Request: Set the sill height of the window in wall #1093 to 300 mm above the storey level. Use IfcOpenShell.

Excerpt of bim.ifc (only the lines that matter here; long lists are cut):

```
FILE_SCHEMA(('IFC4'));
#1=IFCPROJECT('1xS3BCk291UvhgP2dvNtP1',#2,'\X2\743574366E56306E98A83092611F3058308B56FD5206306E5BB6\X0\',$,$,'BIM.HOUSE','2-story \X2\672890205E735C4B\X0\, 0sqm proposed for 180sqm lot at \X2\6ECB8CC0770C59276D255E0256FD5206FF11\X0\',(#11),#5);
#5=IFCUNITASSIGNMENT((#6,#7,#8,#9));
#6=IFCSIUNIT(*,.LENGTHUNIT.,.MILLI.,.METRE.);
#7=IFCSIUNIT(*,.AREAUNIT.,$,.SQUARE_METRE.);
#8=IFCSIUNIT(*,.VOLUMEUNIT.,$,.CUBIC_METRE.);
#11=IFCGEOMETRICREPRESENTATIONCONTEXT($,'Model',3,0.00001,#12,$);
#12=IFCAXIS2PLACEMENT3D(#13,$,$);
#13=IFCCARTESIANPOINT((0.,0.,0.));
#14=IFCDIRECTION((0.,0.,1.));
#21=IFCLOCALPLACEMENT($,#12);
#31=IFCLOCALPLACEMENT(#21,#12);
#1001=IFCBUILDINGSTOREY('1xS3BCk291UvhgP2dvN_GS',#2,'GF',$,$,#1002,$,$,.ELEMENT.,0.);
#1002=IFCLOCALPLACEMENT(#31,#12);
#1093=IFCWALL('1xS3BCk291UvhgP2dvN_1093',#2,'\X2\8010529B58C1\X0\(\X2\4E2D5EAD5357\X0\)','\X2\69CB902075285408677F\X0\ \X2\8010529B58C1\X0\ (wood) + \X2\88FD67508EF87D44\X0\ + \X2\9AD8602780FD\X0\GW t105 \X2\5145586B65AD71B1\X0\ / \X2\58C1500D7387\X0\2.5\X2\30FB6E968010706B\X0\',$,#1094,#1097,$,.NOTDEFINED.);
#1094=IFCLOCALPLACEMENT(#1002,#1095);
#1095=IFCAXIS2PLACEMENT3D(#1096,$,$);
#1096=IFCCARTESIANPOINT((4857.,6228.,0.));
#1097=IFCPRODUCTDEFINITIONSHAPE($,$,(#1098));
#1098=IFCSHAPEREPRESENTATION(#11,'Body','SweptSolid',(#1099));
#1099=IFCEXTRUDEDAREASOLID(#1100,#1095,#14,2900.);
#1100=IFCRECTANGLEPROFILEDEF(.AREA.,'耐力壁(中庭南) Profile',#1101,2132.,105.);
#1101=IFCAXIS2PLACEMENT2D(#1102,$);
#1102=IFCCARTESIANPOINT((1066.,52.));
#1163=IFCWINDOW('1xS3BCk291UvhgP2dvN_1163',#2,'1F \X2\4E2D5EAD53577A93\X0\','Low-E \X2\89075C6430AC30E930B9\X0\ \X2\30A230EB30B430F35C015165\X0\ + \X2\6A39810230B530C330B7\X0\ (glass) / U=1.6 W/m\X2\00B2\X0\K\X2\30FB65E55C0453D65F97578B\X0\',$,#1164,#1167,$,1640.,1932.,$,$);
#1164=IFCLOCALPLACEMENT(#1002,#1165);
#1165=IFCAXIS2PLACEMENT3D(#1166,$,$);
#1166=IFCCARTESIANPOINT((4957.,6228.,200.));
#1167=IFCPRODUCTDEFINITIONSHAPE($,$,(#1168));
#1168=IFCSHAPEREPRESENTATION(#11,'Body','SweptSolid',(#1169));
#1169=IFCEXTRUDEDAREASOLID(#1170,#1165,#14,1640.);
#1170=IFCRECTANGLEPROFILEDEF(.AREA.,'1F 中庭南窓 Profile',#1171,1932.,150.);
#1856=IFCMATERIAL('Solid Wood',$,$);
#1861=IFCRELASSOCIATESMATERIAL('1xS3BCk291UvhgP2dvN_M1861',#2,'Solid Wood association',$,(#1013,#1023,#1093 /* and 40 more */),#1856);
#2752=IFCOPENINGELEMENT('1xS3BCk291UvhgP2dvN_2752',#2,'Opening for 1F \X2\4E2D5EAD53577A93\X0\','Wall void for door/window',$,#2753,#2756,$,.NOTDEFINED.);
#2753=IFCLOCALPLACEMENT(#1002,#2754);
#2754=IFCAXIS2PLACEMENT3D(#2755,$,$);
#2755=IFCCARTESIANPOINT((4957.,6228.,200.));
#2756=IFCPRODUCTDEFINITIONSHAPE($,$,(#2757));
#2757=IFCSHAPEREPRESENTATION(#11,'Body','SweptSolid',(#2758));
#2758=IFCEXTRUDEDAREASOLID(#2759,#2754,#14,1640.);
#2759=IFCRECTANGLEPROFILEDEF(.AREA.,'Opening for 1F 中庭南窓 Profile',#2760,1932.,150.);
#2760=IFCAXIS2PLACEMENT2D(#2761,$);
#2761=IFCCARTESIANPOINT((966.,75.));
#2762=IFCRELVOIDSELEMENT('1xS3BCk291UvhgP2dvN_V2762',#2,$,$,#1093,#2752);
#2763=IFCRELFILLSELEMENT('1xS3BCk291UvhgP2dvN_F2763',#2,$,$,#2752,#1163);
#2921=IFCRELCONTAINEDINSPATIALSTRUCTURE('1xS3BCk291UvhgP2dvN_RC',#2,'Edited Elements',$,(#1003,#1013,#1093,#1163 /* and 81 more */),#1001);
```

```python
import numpy as np
import ifcopenshell
import ifcopenshell.api.geometry
import ifcopenshell.geom
import ifcopenshell.util.element
import ifcopenshell.util.placement
import ifcopenshell.util.shape
import ifcopenshell.util.unit

model = ifcopenshell.open("bim.ifc")
unit_scale = ifcopenshell.util.unit.calculate_unit_scale(model)

window = model.by_id(1163)
opening = window.FillsVoids[0].RelatingOpeningElement
storey = ifcopenshell.util.element.get_container(window, ifc_class="IfcBuildingStorey")
level = ifcopenshell.util.placement.get_local_placement(storey.ObjectPlacement)[2, 3]

# The opening's origin need not be at the sill, so measure its lowest point.
shape = ifcopenshell.geom.create_shape(ifcopenshell.geom.settings(), opening)
bottom = ifcopenshell.util.shape.get_shape_bottom_elevation(shape, shape.geometry) / unit_scale
dz = level + 300.0 - bottom

shift = np.array([0.0, 0.0, dz])
# The window is not placed relative to its opening, so move both.
for product in (opening, window):
    matrix = ifcopenshell.util.placement.get_local_placement(product.ObjectPlacement)
    matrix[:3, 3] += shift
    ifcopenshell.api.geometry.edit_object_placement(model, product=product, matrix=matrix, is_si=False)

print(f"moved by {dz * unit_scale:+.3f} m")

model.write("bim_edited.ifc")
```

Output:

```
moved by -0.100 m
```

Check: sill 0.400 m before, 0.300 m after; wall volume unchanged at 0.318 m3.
